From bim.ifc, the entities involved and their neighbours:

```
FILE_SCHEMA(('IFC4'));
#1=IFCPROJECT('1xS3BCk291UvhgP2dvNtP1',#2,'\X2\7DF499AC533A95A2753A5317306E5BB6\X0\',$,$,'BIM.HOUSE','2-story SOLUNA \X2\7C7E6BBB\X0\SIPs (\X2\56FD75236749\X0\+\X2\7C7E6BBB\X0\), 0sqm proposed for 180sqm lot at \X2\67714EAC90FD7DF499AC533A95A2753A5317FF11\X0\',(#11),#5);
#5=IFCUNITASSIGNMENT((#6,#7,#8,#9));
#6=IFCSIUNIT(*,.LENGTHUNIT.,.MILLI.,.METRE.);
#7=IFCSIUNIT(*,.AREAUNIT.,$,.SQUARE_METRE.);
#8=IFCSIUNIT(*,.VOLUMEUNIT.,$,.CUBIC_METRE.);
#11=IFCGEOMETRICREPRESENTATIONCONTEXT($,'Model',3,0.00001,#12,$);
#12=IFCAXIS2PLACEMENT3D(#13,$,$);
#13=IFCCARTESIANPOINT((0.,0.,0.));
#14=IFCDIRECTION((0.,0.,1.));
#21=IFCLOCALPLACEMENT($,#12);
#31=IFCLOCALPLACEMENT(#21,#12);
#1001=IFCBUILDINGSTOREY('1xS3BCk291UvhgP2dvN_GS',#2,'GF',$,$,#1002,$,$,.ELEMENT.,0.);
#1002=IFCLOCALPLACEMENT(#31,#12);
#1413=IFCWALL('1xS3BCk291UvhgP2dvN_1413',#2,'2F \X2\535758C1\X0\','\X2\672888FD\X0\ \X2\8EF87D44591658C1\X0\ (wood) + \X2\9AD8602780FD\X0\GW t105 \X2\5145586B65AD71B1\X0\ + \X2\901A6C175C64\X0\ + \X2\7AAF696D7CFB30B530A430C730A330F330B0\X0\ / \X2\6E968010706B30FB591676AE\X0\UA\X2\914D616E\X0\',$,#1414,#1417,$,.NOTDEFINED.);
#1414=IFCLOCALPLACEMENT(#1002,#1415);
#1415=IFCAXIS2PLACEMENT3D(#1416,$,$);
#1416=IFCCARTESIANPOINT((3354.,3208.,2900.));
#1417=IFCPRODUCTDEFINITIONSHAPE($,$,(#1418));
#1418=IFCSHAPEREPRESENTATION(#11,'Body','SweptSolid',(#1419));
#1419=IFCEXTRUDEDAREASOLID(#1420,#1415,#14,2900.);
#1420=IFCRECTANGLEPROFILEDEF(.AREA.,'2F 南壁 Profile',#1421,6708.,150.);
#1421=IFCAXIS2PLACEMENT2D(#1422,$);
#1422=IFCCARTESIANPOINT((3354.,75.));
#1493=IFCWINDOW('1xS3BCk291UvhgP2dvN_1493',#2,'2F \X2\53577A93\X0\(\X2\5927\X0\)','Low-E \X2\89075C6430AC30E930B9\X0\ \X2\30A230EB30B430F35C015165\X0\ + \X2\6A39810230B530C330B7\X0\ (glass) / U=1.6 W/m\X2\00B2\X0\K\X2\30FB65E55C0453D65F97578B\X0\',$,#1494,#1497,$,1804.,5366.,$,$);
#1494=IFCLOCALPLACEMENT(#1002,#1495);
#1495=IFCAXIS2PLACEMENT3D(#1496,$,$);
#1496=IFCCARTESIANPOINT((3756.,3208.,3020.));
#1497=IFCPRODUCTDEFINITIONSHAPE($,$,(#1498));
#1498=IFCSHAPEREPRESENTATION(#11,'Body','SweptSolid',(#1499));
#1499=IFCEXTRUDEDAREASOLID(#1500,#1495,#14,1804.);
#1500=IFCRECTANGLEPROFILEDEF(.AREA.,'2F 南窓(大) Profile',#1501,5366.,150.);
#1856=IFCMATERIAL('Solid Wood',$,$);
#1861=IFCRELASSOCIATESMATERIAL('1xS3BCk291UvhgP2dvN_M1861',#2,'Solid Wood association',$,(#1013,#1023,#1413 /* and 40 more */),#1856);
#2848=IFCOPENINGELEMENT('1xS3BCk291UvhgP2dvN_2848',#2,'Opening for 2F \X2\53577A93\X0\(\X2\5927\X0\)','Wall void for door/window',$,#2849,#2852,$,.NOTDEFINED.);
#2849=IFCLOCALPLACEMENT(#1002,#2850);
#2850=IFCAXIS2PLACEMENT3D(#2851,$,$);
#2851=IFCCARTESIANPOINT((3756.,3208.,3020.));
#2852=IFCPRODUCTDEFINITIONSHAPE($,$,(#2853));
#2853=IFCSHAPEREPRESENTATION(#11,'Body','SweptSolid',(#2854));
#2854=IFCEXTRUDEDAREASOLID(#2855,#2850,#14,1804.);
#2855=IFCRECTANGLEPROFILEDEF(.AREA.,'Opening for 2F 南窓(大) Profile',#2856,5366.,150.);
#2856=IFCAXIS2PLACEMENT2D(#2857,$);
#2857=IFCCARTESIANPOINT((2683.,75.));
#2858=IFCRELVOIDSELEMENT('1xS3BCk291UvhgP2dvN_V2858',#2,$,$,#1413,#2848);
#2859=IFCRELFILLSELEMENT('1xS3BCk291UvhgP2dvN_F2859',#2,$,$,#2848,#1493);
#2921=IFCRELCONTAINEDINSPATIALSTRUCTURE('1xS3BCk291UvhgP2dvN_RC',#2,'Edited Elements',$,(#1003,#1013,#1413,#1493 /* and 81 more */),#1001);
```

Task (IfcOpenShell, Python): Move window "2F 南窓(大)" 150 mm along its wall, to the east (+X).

```python
import ifcopenshell
import ifcopenshell.api.geometry
import ifcopenshell.util.placement
import ifcopenshell.util.unit

model = ifcopenshell.open("bim.ifc")
unit_scale = ifcopenshell.util.unit.calculate_unit_scale(model)

window = model.by_id(1493)
opening = window.FillsVoids[0].RelatingOpeningElement
wall = opening.VoidsElements[0].RelatingBuildingElement

wall_matrix = ifcopenshell.util.placement.get_local_placement(wall.ObjectPlacement)
shift = wall_matrix[:3, 0] * 0.15 / unit_scale
before = ifcopenshell.util.placement.get_local_placement(window.ObjectPlacement)[:3, 3].copy()

# The window is not placed relative to its opening, so move both.
for product in (opening, window):
    matrix = ifcopenshell.util.placement.get_local_placement(product.ObjectPlacement)
    matrix[:3, 3] += shift
    ifcopenshell.api.geometry.edit_object_placement(model, product=product, matrix=matrix, is_si=False)

after = ifcopenshell.util.placement.get_local_placement(window.ObjectPlacement)[:3, 3]
print("window moved by", (after - before).round(3) + 0.0)

model.write("bim_rev.ifc")
```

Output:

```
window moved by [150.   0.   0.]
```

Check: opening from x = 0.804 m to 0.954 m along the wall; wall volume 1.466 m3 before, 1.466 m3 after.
